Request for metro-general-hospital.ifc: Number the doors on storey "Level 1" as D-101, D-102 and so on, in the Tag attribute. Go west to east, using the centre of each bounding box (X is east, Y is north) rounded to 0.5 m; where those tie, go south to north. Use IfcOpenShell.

First a look at what the model holds.

```python
import ifcopenshell
import ifcopenshell.util.element
import ifcopenshell.util.placement

model = ifcopenshell.open("metro-general-hospital.ifc")
print(model.schema)
storey = next(s for s in model.by_type("IfcBuildingStorey") if s.Name == "Level 1")
doors = [e for e in ifcopenshell.util.element.get_decomposition(storey) if e.is_a("IfcDoor")]
for e in sorted(doors, key=lambda e: e.id()):
    origin = ifcopenshell.util.placement.get_local_placement(e.ObjectPlacement)[:3, 3]
    print(e.id(), e.Tag, e.Name, origin.round(2) + 0.0, sep=" | ")
```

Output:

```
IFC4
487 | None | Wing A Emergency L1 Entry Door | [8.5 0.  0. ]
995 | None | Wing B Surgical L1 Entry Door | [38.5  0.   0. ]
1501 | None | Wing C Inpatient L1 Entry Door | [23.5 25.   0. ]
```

```python
import ifcopenshell
import ifcopenshell.geom
import ifcopenshell.util.element
import ifcopenshell.util.shape

model = ifcopenshell.open("metro-general-hospital.ifc")
settings = ifcopenshell.geom.settings()
settings.set("use-world-coords", True)


def centre(element):
    shape = ifcopenshell.geom.create_shape(settings, element)
    return ifcopenshell.util.shape.get_bbox_centroid(shape.geometry)


storey = next(s for s in model.by_type("IfcBuildingStorey") if s.Name == "Level 1")
doors = [e for e in ifcopenshell.util.element.get_decomposition(storey) if e.is_a("IfcDoor")]

# Insertion points can sit at a corner or the storey origin, so sort by the geometry (in metres).
centres = {e: centre(e) for e in doors}
doors.sort(key=lambda e: (round(centres[e][0] / 0.5), centres[e][1]))

for i, e in enumerate(doors, start=1):
    number = f"D-1{i:02d}"
    e.Tag = number
    print(e.id(), number)

model.write("metro-general-hospital_edited.ifc")
```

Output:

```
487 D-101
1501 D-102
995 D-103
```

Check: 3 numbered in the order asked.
